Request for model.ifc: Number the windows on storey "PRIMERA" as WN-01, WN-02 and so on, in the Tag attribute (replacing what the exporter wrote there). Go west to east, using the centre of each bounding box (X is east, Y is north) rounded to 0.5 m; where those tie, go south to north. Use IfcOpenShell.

First a look at what the model holds.

```python
import ifcopenshell
import ifcopenshell.util.element
import ifcopenshell.util.placement

model = ifcopenshell.open("model.ifc")
print(model.schema)
storey = next(s for s in model.by_type("IfcBuildingStorey") if s.Name == "PRIMERA")
windows = [e for e in ifcopenshell.util.element.get_decomposition(storey) if e.is_a("IfcWindow")]
for e in sorted(windows, key=lambda e: e.id()):
    origin = ifcopenshell.util.placement.get_local_placement(e.ObjectPlacement)[:3, 3]
    print(e.id(), e.Tag, e.Name, origin.round(2) + 0.0, sep=" | ")
```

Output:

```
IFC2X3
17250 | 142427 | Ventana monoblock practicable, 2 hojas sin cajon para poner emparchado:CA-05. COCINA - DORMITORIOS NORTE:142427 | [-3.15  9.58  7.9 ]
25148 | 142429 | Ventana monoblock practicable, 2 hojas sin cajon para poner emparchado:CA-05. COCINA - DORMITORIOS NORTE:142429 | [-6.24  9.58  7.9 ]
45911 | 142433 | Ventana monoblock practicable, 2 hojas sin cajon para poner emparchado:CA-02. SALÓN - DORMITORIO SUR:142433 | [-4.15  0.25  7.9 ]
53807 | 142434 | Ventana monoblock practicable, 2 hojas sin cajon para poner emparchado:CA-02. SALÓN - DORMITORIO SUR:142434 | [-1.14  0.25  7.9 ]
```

```python
import ifcopenshell
import ifcopenshell.geom
import ifcopenshell.util.element
import ifcopenshell.util.shape

model = ifcopenshell.open("model.ifc")
settings = ifcopenshell.geom.settings()
settings.set("use-world-coords", True)


def centre(element):
    shape = ifcopenshell.geom.create_shape(settings, element)
    return ifcopenshell.util.shape.get_bbox_centroid(shape.geometry)


storey = next(s for s in model.by_type("IfcBuildingStorey") if s.Name == "PRIMERA")
windows = [e for e in ifcopenshell.util.element.get_decomposition(storey) if e.is_a("IfcWindow")]

# Insertion points can sit at a corner or the storey origin, so sort by the geometry (in metres).
centres = {e: centre(e) for e in windows}
windows.sort(key=lambda e: (round(centres[e][0] / 0.5), centres[e][1]))

for i, e in enumerate(windows, start=1):
    number = f"WN-{i:02d}"
    e.Tag = number
    print(e.id(), number)

model.write("model-out.ifc")
```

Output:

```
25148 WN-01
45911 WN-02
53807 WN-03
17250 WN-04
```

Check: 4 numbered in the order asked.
